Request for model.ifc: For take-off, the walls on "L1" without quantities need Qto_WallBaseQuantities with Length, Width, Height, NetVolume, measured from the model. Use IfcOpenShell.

First a look at what the model holds.

```python
import ifcopenshell
import ifcopenshell.util.element
import ifcopenshell.util.unit

model = ifcopenshell.open("model.ifc")
print(model.schema)
for unit_type in ("LENGTHUNIT", "AREAUNIT", "VOLUMEUNIT"):
    print(unit_type, ifcopenshell.util.unit.calculate_unit_scale(model, unit_type))
storey = next(s for s in model.by_type("IfcBuildingStorey") if s.Name == "L1")
walls = [e for e in ifcopenshell.util.element.get_decomposition(storey) if e.is_a("IfcWall")]
for e in sorted(walls, key=lambda e: e.id()):
    print(e.id(), e.is_a(), e.Name, list(ifcopenshell.util.element.get_psets(e, qtos_only=True)), sep=" | ")
```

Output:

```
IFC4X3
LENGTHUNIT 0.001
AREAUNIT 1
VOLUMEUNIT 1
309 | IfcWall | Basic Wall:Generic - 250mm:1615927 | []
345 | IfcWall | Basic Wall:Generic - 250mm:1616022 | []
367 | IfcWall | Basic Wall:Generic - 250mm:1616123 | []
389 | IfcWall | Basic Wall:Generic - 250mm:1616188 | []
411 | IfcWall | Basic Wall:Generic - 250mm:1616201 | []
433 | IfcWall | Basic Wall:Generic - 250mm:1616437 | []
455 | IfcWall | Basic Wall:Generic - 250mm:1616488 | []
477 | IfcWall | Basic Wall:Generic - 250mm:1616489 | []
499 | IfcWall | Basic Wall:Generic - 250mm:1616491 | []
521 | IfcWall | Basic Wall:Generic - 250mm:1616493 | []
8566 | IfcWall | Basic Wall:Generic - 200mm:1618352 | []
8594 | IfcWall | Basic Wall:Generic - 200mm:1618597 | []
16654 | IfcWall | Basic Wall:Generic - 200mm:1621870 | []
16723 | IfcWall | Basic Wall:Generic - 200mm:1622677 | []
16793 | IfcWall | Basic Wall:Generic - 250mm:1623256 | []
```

```python
import ifcopenshell
import ifcopenshell.api.pset
import ifcopenshell.geom
import ifcopenshell.util.element
import ifcopenshell.util.shape
import ifcopenshell.util.unit

model = ifcopenshell.open("model.ifc")
unit_scale = ifcopenshell.util.unit.calculate_unit_scale(model)
volume_scale = ifcopenshell.util.unit.calculate_unit_scale(model, "VOLUMEUNIT")
settings = ifcopenshell.geom.settings()

storey = next(s for s in model.by_type("IfcBuildingStorey") if s.Name == "L1")
walls = [e for e in ifcopenshell.util.element.get_decomposition(storey) if e.is_a("IfcWall")]

for e in sorted(walls, key=lambda e: e.id()):
    if ifcopenshell.util.element.get_psets(e, qtos_only=True, should_inherit=False):
        continue
    # Geometry comes back in metres, in the element's own axes.
    shape = ifcopenshell.geom.create_shape(settings, e)
    values = {
        "Length": ifcopenshell.util.shape.get_x(shape.geometry) / unit_scale,
        "Width": ifcopenshell.util.shape.get_y(shape.geometry) / unit_scale,
        "Height": ifcopenshell.util.shape.get_z(shape.geometry) / unit_scale,
        "NetVolume": ifcopenshell.util.shape.get_volume(shape.geometry) / volume_scale,
    }
    qto = ifcopenshell.api.pset.add_qto(model, product=e, name="Qto_WallBaseQuantities")
    ifcopenshell.api.pset.edit_qto(model, qto=qto, properties=values)
    print(e.id(), {k: round(v, 3) for k, v in values.items()})

model.write("model-out.ifc")
```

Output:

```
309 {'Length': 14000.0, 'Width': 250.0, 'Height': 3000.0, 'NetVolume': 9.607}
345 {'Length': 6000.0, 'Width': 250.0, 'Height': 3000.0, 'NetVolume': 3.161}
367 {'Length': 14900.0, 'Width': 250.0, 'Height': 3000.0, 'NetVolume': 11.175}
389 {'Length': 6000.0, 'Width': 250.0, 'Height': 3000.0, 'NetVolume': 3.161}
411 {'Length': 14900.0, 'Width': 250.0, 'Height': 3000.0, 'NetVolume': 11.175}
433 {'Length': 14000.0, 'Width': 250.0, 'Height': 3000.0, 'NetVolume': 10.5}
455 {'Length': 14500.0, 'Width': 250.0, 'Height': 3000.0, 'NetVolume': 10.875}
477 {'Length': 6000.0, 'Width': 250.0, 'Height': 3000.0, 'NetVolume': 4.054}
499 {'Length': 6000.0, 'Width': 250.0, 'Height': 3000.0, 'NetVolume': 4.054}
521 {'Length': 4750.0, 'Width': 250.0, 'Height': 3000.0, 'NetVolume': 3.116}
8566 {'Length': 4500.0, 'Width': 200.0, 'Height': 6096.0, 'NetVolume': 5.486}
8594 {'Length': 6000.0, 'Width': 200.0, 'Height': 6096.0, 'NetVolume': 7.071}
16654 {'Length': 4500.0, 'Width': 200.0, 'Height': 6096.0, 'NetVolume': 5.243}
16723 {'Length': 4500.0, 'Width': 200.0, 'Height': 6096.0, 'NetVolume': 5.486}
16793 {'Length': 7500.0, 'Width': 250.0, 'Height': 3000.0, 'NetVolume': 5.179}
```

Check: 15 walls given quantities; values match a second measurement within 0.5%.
